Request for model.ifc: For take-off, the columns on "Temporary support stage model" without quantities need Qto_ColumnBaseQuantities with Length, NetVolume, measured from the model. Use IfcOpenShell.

First a look at what the model holds.

```python
import ifcopenshell
import ifcopenshell.util.element
import ifcopenshell.util.unit

model = ifcopenshell.open("model.ifc")
print(model.schema)
for unit_type in ("LENGTHUNIT", "AREAUNIT", "VOLUMEUNIT"):
    print(unit_type, ifcopenshell.util.unit.calculate_unit_scale(model, unit_type))
storey = next(s for s in model.by_type("IfcBuildingStorey") if s.Name == "Temporary support stage model")
columns = [e for e in ifcopenshell.util.element.get_decomposition(storey) if e.is_a("IfcColumn")]
for e in sorted(columns, key=lambda e: e.id()):
    print(e.id(), e.is_a(), e.Name, list(ifcopenshell.util.element.get_psets(e, qtos_only=True)), sep=" | ")
```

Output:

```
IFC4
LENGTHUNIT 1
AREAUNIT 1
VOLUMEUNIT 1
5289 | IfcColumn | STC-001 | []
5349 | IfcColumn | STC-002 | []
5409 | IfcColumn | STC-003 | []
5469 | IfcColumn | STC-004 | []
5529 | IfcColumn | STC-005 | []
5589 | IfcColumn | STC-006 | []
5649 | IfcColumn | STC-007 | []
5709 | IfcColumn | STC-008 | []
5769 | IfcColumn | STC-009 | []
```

```python
import ifcopenshell
import ifcopenshell.api.pset
import ifcopenshell.geom
import ifcopenshell.util.element
import ifcopenshell.util.shape
import ifcopenshell.util.unit

model = ifcopenshell.open("model.ifc")
unit_scale = ifcopenshell.util.unit.calculate_unit_scale(model)
volume_scale = ifcopenshell.util.unit.calculate_unit_scale(model, "VOLUMEUNIT")
settings = ifcopenshell.geom.settings()

storey = next(s for s in model.by_type("IfcBuildingStorey") if s.Name == "Temporary support stage model")
columns = [e for e in ifcopenshell.util.element.get_decomposition(storey) if e.is_a("IfcColumn")]

for e in sorted(columns, key=lambda e: e.id()):
    if ifcopenshell.util.element.get_psets(e, qtos_only=True, should_inherit=False):
        continue
    # Geometry comes back in metres, in the element's own axes.
    shape = ifcopenshell.geom.create_shape(settings, e)
    values = {
        "Length": ifcopenshell.util.shape.get_z(shape.geometry) / unit_scale,
        "NetVolume": ifcopenshell.util.shape.get_volume(shape.geometry) / volume_scale,
    }
    qto = ifcopenshell.api.pset.add_qto(model, product=e, name="Qto_ColumnBaseQuantities")
    ifcopenshell.api.pset.edit_qto(model, qto=qto, properties=values)
    print(e.id(), {k: round(v, 3) for k, v in values.items()})

model.write("model_updated.ifc")
```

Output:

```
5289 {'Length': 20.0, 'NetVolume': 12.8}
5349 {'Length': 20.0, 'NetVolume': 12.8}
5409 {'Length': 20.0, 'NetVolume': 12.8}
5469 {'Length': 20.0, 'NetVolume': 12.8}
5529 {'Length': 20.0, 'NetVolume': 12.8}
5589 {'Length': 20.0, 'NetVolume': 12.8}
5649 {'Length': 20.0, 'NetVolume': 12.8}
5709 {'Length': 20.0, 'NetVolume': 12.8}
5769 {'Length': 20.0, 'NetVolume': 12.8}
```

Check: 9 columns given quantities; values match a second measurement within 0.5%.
